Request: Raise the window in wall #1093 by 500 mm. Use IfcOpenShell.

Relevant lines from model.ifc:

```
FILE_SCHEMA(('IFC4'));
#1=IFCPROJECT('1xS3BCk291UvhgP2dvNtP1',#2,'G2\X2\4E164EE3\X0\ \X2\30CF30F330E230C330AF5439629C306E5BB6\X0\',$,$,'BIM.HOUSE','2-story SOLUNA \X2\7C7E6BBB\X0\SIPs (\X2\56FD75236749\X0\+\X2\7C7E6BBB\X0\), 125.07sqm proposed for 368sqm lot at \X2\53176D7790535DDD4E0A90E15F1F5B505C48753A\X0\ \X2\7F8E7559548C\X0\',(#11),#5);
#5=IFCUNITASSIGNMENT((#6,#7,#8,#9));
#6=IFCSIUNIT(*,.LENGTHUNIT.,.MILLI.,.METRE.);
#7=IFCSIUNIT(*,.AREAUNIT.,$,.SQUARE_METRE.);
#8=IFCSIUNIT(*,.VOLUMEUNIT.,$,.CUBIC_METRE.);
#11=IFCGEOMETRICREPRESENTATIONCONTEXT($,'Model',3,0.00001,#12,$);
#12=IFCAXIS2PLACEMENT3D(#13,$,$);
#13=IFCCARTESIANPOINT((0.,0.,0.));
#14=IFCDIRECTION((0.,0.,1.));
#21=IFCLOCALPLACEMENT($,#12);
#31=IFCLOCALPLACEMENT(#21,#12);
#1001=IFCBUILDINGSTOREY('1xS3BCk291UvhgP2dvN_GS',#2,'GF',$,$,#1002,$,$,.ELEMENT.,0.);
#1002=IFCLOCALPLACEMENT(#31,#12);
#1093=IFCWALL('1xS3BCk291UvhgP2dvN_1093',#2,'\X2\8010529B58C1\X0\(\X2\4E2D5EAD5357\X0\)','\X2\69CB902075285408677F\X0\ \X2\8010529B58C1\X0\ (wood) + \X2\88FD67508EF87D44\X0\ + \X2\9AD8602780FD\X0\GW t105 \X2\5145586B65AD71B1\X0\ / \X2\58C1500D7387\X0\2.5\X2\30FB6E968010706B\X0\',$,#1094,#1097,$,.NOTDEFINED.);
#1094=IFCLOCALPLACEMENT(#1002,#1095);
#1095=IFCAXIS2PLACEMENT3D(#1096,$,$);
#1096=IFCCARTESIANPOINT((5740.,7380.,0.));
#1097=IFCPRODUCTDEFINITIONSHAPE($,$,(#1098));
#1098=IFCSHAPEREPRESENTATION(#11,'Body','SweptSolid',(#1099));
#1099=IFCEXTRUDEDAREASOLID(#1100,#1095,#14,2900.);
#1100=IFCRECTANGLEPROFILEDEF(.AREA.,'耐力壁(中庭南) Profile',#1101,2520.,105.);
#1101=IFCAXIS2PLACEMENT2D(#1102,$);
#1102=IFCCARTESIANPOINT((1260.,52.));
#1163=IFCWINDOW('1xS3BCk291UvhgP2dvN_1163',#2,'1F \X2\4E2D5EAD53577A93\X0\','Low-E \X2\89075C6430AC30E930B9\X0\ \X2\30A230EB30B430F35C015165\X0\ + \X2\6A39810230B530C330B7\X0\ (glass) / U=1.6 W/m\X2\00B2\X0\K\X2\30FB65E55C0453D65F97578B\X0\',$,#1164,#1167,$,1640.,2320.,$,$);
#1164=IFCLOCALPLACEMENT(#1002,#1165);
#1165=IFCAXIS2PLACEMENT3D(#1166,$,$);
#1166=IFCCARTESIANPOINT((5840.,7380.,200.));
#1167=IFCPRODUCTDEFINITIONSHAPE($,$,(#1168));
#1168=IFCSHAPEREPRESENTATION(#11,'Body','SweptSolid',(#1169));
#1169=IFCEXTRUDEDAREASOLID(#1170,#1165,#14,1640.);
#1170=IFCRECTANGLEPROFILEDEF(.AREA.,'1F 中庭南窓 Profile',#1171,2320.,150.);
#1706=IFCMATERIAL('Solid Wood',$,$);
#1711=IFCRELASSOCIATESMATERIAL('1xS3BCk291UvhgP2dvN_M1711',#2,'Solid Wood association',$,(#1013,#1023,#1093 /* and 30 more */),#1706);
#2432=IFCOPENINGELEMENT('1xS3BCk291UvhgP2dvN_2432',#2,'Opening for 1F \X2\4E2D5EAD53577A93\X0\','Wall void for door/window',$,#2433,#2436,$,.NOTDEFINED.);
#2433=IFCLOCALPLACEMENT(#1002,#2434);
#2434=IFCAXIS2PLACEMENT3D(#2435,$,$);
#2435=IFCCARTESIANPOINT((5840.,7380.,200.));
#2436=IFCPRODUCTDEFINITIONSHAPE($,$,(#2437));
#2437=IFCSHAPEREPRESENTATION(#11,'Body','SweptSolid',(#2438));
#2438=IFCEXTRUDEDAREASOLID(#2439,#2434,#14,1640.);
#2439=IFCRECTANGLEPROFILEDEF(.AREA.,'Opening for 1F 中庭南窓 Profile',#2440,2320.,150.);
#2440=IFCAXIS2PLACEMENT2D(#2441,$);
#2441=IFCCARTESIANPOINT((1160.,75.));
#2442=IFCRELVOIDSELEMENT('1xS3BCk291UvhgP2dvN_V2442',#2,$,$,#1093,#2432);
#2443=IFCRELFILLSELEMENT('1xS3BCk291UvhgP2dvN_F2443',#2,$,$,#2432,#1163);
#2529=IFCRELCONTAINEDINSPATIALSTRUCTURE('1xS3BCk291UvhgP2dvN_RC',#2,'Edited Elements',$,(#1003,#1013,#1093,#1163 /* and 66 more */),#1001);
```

```python
import numpy as np
import ifcopenshell
import ifcopenshell.api.geometry
import ifcopenshell.util.placement
import ifcopenshell.util.unit

model = ifcopenshell.open("model.ifc")
unit_scale = ifcopenshell.util.unit.calculate_unit_scale(model)

window = model.by_id(1163)
opening = window.FillsVoids[0].RelatingOpeningElement
dz = 500.0

shift = np.array([0.0, 0.0, dz])
# The window is not placed relative to its opening, so move both.
for product in (opening, window):
    matrix = ifcopenshell.util.placement.get_local_placement(product.ObjectPlacement)
    matrix[:3, 3] += shift
    ifcopenshell.api.geometry.edit_object_placement(model, product=product, matrix=matrix, is_si=False)

print(f"moved by {dz * unit_scale:+.3f} m")

model.write("model_updated.ifc")
```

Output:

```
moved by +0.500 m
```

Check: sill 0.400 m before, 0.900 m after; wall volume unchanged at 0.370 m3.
